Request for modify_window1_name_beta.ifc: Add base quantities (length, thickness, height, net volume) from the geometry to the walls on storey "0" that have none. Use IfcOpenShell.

First a look at what the model holds.

```python
import ifcopenshell
import ifcopenshell.util.element
import ifcopenshell.util.unit

model = ifcopenshell.open("modify_window1_name_beta.ifc")
print(model.schema)
for unit_type in ("LENGTHUNIT", "AREAUNIT", "VOLUMEUNIT"):
    print(unit_type, ifcopenshell.util.unit.calculate_unit_scale(model, unit_type))
storey = next(s for s in model.by_type("IfcBuildingStorey") if s.Name == "0")
walls = [e for e in ifcopenshell.util.element.get_decomposition(storey) if e.is_a("IfcWall")]
for e in sorted(walls, key=lambda e: e.id()):
    print(e.id(), e.is_a(), e.Name, list(ifcopenshell.util.element.get_psets(e, qtos_only=True)), sep=" | ")
```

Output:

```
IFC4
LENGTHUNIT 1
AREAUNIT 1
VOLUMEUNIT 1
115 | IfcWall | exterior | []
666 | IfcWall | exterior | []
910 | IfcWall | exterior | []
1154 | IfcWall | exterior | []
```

```python
import ifcopenshell
import ifcopenshell.api.pset
import ifcopenshell.geom
import ifcopenshell.util.element
import ifcopenshell.util.shape
import ifcopenshell.util.unit

model = ifcopenshell.open("modify_window1_name_beta.ifc")
unit_scale = ifcopenshell.util.unit.calculate_unit_scale(model)
volume_scale = ifcopenshell.util.unit.calculate_unit_scale(model, "VOLUMEUNIT")
settings = ifcopenshell.geom.settings()

storey = next(s for s in model.by_type("IfcBuildingStorey") if s.Name == "0")
walls = [e for e in ifcopenshell.util.element.get_decomposition(storey) if e.is_a("IfcWall")]

for e in sorted(walls, key=lambda e: e.id()):
    if ifcopenshell.util.element.get_psets(e, qtos_only=True, should_inherit=False):
        continue
    # Geometry comes back in metres, in the element's own axes.
    shape = ifcopenshell.geom.create_shape(settings, e)
    values = {
        "Length": ifcopenshell.util.shape.get_x(shape.geometry) / unit_scale,
        "Width": ifcopenshell.util.shape.get_y(shape.geometry) / unit_scale,
        "Height": ifcopenshell.util.shape.get_z(shape.geometry) / unit_scale,
        "NetVolume": ifcopenshell.util.shape.get_volume(shape.geometry) / volume_scale,
    }
    qto = ifcopenshell.api.pset.add_qto(model, product=e, name="Qto_WallBaseQuantities")
    ifcopenshell.api.pset.edit_qto(model, qto=qto, properties=values)
    print(e.id(), {k: round(v, 3) for k, v in values.items()})

model.write("modify_window1_name_beta_rev.ifc")
```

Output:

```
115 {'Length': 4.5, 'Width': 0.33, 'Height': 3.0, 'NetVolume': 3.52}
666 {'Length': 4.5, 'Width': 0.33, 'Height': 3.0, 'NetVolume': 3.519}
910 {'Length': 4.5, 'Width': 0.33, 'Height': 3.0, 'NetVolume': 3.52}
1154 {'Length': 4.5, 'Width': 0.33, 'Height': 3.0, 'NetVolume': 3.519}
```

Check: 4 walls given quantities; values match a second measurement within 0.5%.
